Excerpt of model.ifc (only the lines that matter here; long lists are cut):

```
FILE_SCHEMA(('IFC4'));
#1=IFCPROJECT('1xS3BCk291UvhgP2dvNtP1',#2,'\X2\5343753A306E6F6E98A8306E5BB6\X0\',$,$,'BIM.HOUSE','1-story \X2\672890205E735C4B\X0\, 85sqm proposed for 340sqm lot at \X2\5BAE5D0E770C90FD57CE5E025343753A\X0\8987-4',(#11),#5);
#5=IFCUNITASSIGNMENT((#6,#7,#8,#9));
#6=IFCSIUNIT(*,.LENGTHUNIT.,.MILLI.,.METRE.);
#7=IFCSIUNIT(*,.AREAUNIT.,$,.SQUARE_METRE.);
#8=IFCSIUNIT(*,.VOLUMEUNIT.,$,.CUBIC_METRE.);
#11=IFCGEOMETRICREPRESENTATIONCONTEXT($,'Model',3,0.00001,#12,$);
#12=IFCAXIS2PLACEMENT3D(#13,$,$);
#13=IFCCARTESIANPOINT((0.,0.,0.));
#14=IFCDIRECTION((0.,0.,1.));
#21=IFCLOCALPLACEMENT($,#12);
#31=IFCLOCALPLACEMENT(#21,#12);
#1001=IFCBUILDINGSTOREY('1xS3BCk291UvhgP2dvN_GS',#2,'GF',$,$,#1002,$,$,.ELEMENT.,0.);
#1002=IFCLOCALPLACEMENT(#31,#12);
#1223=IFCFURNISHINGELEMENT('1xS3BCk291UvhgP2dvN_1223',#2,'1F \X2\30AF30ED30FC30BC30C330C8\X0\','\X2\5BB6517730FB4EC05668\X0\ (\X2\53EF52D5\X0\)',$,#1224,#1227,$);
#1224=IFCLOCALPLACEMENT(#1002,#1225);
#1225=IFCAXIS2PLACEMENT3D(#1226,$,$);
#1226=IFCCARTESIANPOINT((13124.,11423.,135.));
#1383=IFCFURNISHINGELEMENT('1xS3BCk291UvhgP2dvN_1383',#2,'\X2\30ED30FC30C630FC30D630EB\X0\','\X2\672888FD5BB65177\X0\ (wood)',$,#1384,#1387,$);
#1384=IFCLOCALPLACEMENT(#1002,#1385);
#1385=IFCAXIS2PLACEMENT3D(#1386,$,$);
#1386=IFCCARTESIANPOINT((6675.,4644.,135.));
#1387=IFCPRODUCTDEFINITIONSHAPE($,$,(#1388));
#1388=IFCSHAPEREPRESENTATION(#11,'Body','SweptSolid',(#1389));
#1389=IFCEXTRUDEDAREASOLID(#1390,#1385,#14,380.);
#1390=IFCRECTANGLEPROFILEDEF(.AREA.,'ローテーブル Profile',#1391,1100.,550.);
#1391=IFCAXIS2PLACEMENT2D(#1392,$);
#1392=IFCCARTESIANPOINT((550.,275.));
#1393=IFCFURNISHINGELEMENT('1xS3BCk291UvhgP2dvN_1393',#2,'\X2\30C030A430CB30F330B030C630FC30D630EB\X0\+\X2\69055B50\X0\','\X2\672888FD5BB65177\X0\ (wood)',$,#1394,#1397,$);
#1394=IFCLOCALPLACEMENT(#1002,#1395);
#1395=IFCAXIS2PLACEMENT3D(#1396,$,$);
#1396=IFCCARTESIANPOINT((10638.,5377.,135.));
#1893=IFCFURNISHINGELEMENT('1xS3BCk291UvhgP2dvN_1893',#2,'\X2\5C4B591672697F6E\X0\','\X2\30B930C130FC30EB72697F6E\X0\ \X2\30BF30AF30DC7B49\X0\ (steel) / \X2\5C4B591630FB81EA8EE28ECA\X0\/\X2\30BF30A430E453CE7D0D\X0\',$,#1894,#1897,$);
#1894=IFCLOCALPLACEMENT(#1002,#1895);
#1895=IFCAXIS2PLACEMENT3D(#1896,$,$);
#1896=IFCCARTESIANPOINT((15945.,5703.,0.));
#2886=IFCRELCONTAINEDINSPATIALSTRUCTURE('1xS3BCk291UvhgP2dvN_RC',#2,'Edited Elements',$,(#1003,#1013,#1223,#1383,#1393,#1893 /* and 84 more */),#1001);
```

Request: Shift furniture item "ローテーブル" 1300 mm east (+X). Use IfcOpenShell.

```python
import ifcopenshell
import ifcopenshell.api.geometry
import ifcopenshell.util.placement

model = ifcopenshell.open("model.ifc")

item = model.by_guid("1xS3BCk291UvhgP2dvN_1383")
matrix = ifcopenshell.util.placement.get_local_placement(item.ObjectPlacement)
matrix[0, 3] += 1300.0
ifcopenshell.api.geometry.edit_object_placement(model, product=item, matrix=matrix, is_si=False)

print(ifcopenshell.util.placement.get_local_placement(item.ObjectPlacement).round(3) + 0.0)

model.write("model_edited.ifc")
```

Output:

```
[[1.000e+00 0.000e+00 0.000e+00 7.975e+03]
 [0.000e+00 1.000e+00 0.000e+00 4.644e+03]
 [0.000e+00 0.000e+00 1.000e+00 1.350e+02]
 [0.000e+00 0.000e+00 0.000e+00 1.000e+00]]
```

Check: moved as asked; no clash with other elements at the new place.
